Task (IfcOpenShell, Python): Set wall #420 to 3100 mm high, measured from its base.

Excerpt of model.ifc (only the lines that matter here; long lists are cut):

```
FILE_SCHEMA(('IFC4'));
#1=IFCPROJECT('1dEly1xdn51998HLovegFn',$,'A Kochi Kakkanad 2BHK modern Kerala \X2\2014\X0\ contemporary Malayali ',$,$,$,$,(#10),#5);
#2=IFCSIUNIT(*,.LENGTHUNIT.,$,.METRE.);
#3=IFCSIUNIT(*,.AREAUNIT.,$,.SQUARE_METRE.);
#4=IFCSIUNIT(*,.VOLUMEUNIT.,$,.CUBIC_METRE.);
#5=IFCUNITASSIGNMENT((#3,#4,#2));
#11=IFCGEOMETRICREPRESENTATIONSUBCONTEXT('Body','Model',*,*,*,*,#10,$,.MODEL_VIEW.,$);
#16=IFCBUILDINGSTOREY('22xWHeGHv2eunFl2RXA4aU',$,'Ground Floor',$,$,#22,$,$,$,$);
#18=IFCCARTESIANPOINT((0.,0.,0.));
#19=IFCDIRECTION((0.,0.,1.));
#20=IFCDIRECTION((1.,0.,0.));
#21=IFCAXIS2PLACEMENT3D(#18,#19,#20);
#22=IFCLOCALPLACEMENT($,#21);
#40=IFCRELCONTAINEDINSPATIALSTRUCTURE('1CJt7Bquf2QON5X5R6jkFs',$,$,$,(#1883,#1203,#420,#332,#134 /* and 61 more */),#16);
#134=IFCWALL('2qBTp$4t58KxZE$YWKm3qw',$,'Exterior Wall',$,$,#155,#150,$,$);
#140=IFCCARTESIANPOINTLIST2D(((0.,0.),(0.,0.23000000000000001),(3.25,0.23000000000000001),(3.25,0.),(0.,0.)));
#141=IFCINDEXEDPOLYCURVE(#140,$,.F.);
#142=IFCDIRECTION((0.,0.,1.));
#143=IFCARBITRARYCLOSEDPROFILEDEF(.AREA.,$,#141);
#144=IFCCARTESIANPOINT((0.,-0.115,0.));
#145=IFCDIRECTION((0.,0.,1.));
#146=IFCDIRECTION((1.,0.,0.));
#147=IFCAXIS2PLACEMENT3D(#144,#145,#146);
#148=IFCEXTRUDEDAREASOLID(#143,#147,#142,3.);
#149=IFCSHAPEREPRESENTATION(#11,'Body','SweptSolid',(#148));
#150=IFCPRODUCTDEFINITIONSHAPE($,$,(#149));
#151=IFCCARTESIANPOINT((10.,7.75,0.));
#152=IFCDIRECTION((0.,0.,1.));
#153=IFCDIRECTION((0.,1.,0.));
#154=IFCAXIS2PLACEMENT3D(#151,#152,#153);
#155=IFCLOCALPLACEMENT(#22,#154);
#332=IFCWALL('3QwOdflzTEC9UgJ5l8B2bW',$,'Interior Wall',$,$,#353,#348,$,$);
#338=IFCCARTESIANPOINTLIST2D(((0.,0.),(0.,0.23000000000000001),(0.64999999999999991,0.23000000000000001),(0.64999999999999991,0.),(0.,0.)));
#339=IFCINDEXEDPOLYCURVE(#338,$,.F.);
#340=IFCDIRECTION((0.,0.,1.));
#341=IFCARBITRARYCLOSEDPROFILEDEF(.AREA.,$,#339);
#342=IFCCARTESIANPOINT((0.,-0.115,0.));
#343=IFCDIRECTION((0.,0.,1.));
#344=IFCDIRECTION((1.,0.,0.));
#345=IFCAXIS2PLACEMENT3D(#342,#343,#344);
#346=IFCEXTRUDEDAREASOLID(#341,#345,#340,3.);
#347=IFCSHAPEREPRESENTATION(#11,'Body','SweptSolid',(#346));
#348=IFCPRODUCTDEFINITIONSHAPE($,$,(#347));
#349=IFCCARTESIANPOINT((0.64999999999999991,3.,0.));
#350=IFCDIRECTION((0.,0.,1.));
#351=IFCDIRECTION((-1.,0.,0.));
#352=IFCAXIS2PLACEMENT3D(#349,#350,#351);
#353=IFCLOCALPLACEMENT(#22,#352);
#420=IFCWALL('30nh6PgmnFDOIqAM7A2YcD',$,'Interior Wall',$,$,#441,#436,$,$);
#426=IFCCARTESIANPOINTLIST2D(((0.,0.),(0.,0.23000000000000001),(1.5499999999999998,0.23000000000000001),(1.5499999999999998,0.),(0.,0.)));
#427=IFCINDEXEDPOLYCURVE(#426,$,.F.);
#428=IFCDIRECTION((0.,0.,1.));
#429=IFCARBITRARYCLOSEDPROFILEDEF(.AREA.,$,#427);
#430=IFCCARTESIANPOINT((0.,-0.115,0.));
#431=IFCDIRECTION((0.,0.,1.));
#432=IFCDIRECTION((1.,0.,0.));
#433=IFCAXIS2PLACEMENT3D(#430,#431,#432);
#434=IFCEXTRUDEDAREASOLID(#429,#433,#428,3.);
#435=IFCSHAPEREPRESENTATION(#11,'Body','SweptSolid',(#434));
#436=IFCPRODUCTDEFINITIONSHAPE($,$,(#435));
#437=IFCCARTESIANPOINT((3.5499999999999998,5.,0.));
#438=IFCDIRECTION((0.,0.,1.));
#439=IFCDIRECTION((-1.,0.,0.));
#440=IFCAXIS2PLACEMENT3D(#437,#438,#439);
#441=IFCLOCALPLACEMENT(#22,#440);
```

```python
import ifcopenshell
import ifcopenshell.geom
import ifcopenshell.util.representation
import ifcopenshell.util.shape
import ifcopenshell.util.unit

model = ifcopenshell.open("model.ifc")
unit_scale = ifcopenshell.util.unit.calculate_unit_scale(model)
settings = ifcopenshell.geom.settings()


def volume(element):
    """Net volume in cubic metres, openings subtracted."""
    shape = ifcopenshell.geom.create_shape(settings, element)
    return ifcopenshell.util.shape.get_volume(shape.geometry)


wall = model.by_id(420)
before = volume(wall)

body = ifcopenshell.util.representation.get_representation(wall, "Model", "Body")
solid = body.Items[0]
old_height = solid.Depth
solid.Depth = 3.1 / unit_scale
after = volume(wall)

print(f"height {old_height:g} -> {solid.Depth:g}, volume {before:.3f} -> {after:.3f} m3")

model.write("model-out.ifc")
```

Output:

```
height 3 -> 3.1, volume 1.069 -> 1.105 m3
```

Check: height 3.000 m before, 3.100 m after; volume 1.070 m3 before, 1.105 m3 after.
